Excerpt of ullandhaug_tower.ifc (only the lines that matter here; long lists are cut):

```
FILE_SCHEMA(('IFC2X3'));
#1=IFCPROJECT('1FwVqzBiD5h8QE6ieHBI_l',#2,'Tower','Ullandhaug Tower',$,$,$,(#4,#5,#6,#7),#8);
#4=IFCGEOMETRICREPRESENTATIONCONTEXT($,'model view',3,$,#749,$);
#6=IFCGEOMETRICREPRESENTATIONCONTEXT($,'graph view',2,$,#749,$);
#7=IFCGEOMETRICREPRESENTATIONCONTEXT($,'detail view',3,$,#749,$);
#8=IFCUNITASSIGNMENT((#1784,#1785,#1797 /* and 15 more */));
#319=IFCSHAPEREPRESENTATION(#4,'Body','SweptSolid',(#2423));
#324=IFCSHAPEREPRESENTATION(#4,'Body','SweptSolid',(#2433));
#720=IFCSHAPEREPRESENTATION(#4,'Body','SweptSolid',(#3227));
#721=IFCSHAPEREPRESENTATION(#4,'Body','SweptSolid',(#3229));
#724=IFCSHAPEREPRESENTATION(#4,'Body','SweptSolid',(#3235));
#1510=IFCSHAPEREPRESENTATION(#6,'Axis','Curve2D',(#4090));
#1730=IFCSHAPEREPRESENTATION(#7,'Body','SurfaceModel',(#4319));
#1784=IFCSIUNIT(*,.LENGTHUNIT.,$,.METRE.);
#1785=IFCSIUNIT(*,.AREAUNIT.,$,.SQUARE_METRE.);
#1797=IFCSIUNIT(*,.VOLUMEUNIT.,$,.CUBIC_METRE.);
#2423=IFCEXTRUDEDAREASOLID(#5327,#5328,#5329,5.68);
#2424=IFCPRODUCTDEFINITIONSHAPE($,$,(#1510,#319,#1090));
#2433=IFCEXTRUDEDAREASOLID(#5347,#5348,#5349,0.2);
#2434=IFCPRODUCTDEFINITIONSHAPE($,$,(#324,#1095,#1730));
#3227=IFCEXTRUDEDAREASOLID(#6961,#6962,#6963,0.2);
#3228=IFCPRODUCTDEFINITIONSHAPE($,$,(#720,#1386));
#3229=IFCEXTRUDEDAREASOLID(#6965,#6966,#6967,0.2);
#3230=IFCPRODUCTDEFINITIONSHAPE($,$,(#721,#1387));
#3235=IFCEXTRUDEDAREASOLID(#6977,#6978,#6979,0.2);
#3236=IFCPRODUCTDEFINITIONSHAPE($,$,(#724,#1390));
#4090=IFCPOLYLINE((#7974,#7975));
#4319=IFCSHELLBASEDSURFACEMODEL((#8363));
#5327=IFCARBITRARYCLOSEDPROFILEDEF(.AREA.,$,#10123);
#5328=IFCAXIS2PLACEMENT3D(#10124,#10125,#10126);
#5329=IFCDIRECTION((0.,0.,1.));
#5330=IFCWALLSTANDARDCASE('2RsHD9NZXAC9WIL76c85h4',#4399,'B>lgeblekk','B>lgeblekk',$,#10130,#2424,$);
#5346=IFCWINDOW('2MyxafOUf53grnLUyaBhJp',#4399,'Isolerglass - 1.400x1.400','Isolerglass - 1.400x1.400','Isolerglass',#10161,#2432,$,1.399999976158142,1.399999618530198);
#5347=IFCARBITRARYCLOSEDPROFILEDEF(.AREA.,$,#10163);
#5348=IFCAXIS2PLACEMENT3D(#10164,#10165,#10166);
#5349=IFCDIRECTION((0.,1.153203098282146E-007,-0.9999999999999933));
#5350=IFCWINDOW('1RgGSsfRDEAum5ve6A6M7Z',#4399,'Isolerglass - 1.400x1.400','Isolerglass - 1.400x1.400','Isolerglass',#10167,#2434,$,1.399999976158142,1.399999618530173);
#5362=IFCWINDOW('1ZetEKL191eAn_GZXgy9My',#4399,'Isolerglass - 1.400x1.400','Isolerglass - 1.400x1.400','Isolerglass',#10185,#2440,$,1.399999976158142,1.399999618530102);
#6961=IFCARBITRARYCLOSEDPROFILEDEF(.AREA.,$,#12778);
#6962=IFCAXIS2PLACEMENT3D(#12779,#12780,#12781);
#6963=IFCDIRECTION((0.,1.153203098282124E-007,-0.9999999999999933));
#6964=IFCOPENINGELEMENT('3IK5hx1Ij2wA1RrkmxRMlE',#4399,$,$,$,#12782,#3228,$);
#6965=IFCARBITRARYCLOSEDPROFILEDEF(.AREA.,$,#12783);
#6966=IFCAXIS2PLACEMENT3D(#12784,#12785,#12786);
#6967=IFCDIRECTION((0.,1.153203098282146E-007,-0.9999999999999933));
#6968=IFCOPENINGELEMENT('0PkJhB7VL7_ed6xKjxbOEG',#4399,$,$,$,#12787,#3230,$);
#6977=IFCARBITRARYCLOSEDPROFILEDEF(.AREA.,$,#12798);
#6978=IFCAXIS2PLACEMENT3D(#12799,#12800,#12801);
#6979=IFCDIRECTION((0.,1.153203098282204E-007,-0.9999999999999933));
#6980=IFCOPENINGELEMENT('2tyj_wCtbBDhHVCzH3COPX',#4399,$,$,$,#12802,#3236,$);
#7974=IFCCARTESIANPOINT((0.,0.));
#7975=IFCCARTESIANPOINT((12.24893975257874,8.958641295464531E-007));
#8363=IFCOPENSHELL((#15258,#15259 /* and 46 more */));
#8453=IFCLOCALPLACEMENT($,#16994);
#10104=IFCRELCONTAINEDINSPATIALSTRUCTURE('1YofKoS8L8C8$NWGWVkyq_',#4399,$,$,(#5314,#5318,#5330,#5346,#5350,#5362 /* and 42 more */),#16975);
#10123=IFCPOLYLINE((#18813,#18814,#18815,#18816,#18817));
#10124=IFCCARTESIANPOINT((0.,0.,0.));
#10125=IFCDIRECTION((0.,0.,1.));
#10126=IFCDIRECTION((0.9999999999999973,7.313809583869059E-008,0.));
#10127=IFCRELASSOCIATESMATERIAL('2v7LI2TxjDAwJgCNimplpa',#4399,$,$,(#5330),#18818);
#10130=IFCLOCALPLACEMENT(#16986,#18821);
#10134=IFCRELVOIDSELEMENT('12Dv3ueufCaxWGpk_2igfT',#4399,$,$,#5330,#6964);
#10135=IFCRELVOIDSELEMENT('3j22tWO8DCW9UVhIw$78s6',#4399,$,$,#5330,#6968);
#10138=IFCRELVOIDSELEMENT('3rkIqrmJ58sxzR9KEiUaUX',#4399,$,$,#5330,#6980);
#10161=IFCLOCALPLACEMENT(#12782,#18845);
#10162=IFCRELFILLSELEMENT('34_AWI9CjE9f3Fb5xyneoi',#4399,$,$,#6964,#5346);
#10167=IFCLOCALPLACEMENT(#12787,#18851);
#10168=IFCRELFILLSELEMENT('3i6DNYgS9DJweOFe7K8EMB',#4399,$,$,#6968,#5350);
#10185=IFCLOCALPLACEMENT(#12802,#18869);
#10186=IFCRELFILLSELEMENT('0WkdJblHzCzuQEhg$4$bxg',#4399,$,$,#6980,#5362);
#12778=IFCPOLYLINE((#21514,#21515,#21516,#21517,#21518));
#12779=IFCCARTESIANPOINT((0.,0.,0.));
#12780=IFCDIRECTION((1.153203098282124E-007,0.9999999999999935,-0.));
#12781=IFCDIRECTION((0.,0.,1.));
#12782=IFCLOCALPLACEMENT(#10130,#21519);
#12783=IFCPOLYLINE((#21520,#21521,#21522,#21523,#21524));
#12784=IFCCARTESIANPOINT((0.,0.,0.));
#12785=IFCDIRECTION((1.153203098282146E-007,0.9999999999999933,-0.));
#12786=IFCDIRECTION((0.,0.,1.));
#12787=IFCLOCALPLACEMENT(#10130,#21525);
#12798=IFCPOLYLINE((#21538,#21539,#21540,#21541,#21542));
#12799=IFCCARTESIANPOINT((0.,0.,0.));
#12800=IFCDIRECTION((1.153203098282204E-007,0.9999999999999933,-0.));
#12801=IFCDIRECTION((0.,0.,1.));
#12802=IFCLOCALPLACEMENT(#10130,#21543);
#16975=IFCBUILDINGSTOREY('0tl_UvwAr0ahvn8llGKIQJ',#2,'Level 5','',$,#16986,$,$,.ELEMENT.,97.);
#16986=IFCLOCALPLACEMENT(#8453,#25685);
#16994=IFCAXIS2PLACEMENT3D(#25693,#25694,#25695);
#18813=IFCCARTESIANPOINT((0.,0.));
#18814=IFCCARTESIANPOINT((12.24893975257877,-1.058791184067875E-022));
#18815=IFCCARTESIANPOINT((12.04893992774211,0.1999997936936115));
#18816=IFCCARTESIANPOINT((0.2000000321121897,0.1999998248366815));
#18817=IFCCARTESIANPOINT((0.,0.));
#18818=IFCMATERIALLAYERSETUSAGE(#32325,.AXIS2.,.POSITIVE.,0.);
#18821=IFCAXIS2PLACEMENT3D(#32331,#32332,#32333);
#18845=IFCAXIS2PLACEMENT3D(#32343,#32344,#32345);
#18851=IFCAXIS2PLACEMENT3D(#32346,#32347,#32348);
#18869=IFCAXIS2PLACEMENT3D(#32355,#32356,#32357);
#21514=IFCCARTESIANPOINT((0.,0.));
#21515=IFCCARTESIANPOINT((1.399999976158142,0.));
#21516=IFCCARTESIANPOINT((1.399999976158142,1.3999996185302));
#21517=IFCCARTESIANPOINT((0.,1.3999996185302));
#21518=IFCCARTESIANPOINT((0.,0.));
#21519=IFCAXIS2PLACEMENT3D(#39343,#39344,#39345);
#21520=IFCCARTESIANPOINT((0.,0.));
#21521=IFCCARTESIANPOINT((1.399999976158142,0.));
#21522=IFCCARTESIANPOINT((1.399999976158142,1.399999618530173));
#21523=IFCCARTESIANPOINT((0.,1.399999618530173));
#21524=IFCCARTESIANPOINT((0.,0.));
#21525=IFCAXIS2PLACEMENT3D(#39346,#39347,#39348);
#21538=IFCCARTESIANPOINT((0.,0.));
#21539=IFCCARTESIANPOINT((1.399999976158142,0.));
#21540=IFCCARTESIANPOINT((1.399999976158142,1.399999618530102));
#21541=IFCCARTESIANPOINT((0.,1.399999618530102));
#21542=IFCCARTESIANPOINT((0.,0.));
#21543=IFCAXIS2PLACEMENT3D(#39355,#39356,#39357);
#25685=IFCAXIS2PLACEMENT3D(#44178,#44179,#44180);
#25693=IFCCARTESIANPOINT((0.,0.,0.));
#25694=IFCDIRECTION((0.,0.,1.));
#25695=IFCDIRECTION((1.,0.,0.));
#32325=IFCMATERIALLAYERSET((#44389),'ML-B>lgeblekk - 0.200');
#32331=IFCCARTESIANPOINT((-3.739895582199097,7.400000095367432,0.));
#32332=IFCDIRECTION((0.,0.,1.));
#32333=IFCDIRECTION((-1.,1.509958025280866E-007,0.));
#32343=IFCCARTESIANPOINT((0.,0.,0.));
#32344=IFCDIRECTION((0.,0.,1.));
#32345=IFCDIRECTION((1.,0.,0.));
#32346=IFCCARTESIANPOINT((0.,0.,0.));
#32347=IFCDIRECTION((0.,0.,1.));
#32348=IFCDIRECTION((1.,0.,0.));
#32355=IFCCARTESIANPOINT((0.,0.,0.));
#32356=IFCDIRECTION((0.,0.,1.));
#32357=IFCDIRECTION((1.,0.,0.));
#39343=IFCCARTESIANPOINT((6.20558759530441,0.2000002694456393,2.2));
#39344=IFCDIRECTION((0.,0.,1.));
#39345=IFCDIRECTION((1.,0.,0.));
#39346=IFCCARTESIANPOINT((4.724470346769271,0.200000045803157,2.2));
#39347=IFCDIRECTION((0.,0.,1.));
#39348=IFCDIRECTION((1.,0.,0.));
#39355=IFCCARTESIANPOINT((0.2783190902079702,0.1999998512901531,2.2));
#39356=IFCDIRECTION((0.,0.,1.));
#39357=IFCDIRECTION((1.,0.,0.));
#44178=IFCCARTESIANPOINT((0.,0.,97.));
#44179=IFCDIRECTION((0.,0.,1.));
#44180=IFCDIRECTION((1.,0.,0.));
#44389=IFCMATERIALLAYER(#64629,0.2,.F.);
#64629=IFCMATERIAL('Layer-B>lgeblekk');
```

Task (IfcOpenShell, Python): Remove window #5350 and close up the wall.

```python
import ifcopenshell
import ifcopenshell.api.feature
import ifcopenshell.api.root
import ifcopenshell.geom
import ifcopenshell.util.shape

model = ifcopenshell.open("ullandhaug_tower.ifc")
settings = ifcopenshell.geom.settings()


def volume(element):
    """Net volume in cubic metres, openings subtracted."""
    shape = ifcopenshell.geom.create_shape(settings, element)
    return ifcopenshell.util.shape.get_volume(shape.geometry)


window = model.by_guid("1RgGSsfRDEAum5ve6A6M7Z")
opening = window.FillsVoids[0].RelatingOpeningElement
wall = opening.VoidsElements[0].RelatingBuildingElement
before = volume(wall)

ifcopenshell.api.root.remove_product(model, product=window)
ifcopenshell.api.feature.remove_feature(model, feature=opening)

after = volume(wall)

print(f"wall volume {before:.3f} -> {after:.3f} m3")

model.write("ullandhaug_tower_updated.ifc")
```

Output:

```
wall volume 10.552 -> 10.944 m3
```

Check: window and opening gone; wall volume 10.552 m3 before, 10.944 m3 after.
